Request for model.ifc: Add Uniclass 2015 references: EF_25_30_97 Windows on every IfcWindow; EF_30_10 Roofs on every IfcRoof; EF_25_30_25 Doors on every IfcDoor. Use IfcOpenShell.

First a look at what the model holds.

```python
import ifcopenshell

model = ifcopenshell.open("model.ifc")
print(model.schema)
print("classifications:", [c.Name for c in model.by_type("IfcClassification")])
for ifc_class in ("IfcDoor", "IfcRoof", "IfcStair", "IfcWall", "IfcWindow"):
    print(ifc_class, len(model.by_type(ifc_class)))
```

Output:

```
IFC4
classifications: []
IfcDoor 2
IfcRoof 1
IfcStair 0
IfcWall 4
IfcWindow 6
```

```python
import ifcopenshell
import ifcopenshell.api.classification

model = ifcopenshell.open("model.ifc")

system = ifcopenshell.api.classification.add_classification(model, classification="Uniclass 2015")

codes = {
    "IfcWindow": ("EF_25_30_97", "Windows"),
    "IfcRoof": ("EF_30_10", "Roofs"),
    "IfcDoor": ("EF_25_30_25", "Doors"),
}
for ifc_class, (code, name) in codes.items():
    products = model.by_type(ifc_class)
    ifcopenshell.api.classification.add_reference(
        model, products=products, classification=system, identification=code, name=name
    )
    print(code, len(products))

model.write("model-out.ifc")
```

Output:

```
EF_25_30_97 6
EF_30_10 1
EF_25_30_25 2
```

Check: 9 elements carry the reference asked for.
